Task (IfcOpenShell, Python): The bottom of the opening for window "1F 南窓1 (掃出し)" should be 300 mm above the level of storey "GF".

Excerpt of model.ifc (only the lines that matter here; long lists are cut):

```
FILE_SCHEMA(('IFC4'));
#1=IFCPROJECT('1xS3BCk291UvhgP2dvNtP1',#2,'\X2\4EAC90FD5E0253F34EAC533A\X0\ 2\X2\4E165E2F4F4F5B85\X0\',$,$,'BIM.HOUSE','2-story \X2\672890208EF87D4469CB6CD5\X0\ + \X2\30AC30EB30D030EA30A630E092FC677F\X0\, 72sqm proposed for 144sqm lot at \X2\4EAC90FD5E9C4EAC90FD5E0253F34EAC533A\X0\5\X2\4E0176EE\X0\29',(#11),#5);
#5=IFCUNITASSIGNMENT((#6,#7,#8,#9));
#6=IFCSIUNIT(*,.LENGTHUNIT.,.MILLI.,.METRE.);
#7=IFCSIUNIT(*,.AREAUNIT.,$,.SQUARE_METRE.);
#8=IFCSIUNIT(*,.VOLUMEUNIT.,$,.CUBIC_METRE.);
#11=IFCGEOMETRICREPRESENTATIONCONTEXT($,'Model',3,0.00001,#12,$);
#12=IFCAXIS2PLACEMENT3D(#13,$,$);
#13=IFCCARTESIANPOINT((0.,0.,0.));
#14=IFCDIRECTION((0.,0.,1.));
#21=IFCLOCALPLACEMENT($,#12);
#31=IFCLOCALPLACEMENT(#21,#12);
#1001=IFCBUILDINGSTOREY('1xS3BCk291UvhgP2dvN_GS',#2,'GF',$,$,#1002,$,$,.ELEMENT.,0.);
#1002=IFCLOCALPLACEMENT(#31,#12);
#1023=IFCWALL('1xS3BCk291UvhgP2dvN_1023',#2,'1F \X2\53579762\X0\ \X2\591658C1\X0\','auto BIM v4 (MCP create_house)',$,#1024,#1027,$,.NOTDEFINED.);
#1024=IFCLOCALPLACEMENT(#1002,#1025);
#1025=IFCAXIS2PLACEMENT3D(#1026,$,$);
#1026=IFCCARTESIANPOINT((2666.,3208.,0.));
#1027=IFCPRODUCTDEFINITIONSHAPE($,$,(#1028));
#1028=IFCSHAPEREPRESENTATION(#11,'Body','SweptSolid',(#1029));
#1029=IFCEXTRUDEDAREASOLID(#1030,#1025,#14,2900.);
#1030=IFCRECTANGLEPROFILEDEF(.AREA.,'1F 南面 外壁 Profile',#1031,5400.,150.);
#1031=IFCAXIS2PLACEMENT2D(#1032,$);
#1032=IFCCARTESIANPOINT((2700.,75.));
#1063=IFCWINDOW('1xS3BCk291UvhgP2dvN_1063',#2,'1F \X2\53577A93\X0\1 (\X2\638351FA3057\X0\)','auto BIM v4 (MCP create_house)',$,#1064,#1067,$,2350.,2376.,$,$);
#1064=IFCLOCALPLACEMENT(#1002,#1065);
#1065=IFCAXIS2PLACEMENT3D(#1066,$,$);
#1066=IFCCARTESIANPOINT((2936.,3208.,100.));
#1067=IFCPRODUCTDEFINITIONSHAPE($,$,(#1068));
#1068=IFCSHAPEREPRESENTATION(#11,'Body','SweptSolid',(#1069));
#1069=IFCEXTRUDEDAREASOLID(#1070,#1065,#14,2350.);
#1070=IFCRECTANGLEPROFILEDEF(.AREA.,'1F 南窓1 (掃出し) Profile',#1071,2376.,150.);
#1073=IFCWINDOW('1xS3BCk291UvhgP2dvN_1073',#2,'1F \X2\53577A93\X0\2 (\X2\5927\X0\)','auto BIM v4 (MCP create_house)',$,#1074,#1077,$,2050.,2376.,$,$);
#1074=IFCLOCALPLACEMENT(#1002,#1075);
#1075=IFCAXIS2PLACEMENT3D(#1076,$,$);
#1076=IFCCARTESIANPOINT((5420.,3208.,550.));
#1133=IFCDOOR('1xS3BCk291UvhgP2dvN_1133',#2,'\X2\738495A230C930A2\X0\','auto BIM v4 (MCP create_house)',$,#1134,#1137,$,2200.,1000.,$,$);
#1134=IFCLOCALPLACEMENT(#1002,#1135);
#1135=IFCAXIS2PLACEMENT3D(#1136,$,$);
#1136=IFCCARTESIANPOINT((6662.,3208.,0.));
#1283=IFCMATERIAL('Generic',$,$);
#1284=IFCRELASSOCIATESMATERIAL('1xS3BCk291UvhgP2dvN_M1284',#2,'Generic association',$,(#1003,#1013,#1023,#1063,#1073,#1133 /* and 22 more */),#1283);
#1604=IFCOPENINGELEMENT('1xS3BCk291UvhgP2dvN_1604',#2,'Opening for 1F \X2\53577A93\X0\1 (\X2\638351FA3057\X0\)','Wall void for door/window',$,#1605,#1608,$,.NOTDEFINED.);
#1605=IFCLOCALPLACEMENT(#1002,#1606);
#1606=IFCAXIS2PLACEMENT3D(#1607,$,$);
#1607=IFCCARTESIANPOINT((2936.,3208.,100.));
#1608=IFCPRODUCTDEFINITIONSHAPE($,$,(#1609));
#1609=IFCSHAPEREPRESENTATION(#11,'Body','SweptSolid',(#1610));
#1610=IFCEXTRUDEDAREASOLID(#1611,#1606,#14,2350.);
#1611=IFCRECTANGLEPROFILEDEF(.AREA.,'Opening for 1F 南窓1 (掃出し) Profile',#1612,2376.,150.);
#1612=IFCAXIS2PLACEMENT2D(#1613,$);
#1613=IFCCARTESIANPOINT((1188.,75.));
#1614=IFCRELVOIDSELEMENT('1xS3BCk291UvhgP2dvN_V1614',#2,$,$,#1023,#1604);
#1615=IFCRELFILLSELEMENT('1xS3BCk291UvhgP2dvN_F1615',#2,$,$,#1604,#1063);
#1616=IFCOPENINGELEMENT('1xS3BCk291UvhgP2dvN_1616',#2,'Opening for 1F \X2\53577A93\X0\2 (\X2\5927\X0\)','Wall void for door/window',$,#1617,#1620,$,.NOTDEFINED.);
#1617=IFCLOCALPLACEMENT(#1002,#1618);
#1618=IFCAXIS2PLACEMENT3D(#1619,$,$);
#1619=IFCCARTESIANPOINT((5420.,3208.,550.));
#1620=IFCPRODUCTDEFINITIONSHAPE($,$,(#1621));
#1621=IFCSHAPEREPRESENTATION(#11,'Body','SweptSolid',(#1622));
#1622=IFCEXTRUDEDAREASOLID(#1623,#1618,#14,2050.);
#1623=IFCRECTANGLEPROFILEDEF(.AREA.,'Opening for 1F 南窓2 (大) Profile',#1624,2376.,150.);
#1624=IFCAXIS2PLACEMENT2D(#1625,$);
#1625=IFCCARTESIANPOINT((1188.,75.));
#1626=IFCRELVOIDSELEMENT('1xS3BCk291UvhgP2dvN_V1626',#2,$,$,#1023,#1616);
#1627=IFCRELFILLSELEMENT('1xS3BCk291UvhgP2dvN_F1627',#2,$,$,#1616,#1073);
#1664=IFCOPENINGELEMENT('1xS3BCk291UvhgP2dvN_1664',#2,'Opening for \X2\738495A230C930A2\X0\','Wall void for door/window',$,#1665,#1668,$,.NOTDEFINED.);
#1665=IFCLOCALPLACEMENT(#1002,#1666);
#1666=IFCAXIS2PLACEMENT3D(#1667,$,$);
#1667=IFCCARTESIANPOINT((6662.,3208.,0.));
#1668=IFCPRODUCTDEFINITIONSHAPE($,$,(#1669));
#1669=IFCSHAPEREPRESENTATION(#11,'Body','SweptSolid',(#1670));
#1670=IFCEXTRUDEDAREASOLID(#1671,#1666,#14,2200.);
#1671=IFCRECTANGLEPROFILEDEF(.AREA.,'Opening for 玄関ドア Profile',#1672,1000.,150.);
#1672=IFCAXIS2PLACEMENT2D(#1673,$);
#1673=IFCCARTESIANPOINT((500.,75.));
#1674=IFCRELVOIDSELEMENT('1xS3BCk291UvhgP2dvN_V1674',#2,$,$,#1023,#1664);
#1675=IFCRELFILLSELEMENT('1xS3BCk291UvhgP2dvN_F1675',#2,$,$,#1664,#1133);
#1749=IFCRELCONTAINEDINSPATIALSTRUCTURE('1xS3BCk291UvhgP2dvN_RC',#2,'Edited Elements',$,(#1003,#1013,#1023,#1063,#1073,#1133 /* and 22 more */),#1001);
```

```python
import numpy as np
import ifcopenshell
import ifcopenshell.api.geometry
import ifcopenshell.geom
import ifcopenshell.util.element
import ifcopenshell.util.placement
import ifcopenshell.util.shape
import ifcopenshell.util.unit

model = ifcopenshell.open("model.ifc")
unit_scale = ifcopenshell.util.unit.calculate_unit_scale(model)

window = model.by_guid("1xS3BCk291UvhgP2dvN_1063")
opening = window.FillsVoids[0].RelatingOpeningElement
storey = ifcopenshell.util.element.get_container(window, ifc_class="IfcBuildingStorey")
level = ifcopenshell.util.placement.get_local_placement(storey.ObjectPlacement)[2, 3]

# The opening's origin need not be at the sill, so measure its lowest point.
shape = ifcopenshell.geom.create_shape(ifcopenshell.geom.settings(), opening)
bottom = ifcopenshell.util.shape.get_shape_bottom_elevation(shape, shape.geometry) / unit_scale
dz = level + 0.3 / unit_scale - bottom

shift = np.array([0.0, 0.0, dz])
# The window is not placed relative to its opening, so move both.
for product in (opening, window):
    matrix = ifcopenshell.util.placement.get_local_placement(product.ObjectPlacement)
    matrix[:3, 3] += shift
    ifcopenshell.api.geometry.edit_object_placement(model, product=product, matrix=matrix, is_si=False)

print(f"moved by {dz * unit_scale:+.3f} m")

model.write("model_updated.ifc")
```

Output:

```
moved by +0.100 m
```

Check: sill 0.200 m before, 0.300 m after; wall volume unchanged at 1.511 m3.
